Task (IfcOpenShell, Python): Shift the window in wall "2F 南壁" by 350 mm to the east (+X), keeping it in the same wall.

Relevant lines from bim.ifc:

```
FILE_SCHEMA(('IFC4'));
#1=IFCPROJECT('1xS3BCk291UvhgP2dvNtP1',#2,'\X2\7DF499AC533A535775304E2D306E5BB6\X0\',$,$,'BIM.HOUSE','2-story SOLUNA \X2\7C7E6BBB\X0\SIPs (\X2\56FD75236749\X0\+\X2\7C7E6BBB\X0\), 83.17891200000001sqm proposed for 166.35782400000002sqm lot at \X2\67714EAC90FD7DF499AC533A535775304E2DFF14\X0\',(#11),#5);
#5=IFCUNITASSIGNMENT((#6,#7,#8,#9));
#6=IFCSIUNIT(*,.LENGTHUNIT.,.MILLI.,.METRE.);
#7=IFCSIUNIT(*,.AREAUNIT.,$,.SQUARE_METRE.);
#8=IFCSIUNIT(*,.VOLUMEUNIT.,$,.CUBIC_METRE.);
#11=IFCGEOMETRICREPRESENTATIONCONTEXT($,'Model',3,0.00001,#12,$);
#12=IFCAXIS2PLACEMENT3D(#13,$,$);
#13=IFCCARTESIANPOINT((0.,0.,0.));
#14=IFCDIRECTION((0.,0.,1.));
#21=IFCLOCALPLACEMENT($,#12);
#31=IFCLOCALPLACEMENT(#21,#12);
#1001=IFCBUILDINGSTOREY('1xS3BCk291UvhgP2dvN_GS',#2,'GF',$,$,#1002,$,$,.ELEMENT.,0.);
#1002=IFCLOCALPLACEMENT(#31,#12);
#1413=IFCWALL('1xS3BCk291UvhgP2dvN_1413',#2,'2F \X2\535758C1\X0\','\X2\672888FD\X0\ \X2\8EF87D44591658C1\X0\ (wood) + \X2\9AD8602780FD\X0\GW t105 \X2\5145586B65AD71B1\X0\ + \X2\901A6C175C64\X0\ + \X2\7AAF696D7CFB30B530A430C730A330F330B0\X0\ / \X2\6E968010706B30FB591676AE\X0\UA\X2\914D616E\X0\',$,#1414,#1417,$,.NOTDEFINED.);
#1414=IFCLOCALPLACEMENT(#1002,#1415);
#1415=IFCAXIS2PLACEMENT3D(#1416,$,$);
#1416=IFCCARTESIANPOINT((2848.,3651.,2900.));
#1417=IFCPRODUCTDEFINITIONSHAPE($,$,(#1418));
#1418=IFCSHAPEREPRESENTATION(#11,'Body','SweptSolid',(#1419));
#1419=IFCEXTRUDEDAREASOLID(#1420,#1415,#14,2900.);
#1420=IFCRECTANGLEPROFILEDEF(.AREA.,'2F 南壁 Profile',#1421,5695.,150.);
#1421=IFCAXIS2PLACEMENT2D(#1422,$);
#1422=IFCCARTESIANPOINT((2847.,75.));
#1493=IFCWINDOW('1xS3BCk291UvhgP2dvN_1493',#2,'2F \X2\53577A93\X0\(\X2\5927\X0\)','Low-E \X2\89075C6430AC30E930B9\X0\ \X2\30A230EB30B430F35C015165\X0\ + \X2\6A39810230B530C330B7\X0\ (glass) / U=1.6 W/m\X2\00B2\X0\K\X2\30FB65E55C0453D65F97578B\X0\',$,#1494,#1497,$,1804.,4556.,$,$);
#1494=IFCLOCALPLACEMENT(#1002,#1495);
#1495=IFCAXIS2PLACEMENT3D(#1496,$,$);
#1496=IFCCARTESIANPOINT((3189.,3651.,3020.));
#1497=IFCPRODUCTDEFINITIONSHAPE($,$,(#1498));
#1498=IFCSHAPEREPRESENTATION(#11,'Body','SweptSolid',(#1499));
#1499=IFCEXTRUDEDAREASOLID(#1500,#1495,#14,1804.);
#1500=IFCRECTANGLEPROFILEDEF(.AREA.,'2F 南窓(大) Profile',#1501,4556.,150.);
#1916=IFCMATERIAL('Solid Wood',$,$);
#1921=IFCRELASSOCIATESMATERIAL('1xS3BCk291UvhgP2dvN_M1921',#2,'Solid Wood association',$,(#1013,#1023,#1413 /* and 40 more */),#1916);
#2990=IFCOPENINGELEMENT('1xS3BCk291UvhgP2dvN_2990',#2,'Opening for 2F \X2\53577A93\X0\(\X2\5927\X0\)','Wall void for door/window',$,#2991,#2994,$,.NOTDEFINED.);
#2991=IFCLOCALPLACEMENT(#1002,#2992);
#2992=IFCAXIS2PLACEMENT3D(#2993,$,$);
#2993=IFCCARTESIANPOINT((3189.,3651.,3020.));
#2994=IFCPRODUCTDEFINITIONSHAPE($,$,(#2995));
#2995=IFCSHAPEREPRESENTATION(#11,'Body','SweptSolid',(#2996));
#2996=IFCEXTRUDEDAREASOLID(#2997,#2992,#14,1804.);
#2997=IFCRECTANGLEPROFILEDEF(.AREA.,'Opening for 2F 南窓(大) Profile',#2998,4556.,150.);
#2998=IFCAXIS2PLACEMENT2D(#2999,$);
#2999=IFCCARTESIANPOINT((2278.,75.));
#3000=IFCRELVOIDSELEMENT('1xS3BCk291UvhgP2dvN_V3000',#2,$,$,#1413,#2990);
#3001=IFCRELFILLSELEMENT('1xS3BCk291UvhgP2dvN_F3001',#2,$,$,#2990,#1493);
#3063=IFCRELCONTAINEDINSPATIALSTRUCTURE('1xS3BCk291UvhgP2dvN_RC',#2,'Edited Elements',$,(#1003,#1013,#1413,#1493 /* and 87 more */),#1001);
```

```python
import ifcopenshell
import ifcopenshell.api.geometry
import ifcopenshell.util.placement
import ifcopenshell.util.unit

model = ifcopenshell.open("bim.ifc")
unit_scale = ifcopenshell.util.unit.calculate_unit_scale(model)

window = model.by_guid("1xS3BCk291UvhgP2dvN_1493")
opening = window.FillsVoids[0].RelatingOpeningElement
wall = opening.VoidsElements[0].RelatingBuildingElement

wall_matrix = ifcopenshell.util.placement.get_local_placement(wall.ObjectPlacement)
shift = wall_matrix[:3, 0] * 0.35 / unit_scale
before = ifcopenshell.util.placement.get_local_placement(window.ObjectPlacement)[:3, 3].copy()

# The window is not placed relative to its opening, so move both.
for product in (opening, window):
    matrix = ifcopenshell.util.placement.get_local_placement(product.ObjectPlacement)
    matrix[:3, 3] += shift
    ifcopenshell.api.geometry.edit_object_placement(model, product=product, matrix=matrix, is_si=False)

after = ifcopenshell.util.placement.get_local_placement(window.ObjectPlacement)[:3, 3]
print("window moved by", (after - before).round(3) + 0.0)

model.write("bim_updated.ifc")
```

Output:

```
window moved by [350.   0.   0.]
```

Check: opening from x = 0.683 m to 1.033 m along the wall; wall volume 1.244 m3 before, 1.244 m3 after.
